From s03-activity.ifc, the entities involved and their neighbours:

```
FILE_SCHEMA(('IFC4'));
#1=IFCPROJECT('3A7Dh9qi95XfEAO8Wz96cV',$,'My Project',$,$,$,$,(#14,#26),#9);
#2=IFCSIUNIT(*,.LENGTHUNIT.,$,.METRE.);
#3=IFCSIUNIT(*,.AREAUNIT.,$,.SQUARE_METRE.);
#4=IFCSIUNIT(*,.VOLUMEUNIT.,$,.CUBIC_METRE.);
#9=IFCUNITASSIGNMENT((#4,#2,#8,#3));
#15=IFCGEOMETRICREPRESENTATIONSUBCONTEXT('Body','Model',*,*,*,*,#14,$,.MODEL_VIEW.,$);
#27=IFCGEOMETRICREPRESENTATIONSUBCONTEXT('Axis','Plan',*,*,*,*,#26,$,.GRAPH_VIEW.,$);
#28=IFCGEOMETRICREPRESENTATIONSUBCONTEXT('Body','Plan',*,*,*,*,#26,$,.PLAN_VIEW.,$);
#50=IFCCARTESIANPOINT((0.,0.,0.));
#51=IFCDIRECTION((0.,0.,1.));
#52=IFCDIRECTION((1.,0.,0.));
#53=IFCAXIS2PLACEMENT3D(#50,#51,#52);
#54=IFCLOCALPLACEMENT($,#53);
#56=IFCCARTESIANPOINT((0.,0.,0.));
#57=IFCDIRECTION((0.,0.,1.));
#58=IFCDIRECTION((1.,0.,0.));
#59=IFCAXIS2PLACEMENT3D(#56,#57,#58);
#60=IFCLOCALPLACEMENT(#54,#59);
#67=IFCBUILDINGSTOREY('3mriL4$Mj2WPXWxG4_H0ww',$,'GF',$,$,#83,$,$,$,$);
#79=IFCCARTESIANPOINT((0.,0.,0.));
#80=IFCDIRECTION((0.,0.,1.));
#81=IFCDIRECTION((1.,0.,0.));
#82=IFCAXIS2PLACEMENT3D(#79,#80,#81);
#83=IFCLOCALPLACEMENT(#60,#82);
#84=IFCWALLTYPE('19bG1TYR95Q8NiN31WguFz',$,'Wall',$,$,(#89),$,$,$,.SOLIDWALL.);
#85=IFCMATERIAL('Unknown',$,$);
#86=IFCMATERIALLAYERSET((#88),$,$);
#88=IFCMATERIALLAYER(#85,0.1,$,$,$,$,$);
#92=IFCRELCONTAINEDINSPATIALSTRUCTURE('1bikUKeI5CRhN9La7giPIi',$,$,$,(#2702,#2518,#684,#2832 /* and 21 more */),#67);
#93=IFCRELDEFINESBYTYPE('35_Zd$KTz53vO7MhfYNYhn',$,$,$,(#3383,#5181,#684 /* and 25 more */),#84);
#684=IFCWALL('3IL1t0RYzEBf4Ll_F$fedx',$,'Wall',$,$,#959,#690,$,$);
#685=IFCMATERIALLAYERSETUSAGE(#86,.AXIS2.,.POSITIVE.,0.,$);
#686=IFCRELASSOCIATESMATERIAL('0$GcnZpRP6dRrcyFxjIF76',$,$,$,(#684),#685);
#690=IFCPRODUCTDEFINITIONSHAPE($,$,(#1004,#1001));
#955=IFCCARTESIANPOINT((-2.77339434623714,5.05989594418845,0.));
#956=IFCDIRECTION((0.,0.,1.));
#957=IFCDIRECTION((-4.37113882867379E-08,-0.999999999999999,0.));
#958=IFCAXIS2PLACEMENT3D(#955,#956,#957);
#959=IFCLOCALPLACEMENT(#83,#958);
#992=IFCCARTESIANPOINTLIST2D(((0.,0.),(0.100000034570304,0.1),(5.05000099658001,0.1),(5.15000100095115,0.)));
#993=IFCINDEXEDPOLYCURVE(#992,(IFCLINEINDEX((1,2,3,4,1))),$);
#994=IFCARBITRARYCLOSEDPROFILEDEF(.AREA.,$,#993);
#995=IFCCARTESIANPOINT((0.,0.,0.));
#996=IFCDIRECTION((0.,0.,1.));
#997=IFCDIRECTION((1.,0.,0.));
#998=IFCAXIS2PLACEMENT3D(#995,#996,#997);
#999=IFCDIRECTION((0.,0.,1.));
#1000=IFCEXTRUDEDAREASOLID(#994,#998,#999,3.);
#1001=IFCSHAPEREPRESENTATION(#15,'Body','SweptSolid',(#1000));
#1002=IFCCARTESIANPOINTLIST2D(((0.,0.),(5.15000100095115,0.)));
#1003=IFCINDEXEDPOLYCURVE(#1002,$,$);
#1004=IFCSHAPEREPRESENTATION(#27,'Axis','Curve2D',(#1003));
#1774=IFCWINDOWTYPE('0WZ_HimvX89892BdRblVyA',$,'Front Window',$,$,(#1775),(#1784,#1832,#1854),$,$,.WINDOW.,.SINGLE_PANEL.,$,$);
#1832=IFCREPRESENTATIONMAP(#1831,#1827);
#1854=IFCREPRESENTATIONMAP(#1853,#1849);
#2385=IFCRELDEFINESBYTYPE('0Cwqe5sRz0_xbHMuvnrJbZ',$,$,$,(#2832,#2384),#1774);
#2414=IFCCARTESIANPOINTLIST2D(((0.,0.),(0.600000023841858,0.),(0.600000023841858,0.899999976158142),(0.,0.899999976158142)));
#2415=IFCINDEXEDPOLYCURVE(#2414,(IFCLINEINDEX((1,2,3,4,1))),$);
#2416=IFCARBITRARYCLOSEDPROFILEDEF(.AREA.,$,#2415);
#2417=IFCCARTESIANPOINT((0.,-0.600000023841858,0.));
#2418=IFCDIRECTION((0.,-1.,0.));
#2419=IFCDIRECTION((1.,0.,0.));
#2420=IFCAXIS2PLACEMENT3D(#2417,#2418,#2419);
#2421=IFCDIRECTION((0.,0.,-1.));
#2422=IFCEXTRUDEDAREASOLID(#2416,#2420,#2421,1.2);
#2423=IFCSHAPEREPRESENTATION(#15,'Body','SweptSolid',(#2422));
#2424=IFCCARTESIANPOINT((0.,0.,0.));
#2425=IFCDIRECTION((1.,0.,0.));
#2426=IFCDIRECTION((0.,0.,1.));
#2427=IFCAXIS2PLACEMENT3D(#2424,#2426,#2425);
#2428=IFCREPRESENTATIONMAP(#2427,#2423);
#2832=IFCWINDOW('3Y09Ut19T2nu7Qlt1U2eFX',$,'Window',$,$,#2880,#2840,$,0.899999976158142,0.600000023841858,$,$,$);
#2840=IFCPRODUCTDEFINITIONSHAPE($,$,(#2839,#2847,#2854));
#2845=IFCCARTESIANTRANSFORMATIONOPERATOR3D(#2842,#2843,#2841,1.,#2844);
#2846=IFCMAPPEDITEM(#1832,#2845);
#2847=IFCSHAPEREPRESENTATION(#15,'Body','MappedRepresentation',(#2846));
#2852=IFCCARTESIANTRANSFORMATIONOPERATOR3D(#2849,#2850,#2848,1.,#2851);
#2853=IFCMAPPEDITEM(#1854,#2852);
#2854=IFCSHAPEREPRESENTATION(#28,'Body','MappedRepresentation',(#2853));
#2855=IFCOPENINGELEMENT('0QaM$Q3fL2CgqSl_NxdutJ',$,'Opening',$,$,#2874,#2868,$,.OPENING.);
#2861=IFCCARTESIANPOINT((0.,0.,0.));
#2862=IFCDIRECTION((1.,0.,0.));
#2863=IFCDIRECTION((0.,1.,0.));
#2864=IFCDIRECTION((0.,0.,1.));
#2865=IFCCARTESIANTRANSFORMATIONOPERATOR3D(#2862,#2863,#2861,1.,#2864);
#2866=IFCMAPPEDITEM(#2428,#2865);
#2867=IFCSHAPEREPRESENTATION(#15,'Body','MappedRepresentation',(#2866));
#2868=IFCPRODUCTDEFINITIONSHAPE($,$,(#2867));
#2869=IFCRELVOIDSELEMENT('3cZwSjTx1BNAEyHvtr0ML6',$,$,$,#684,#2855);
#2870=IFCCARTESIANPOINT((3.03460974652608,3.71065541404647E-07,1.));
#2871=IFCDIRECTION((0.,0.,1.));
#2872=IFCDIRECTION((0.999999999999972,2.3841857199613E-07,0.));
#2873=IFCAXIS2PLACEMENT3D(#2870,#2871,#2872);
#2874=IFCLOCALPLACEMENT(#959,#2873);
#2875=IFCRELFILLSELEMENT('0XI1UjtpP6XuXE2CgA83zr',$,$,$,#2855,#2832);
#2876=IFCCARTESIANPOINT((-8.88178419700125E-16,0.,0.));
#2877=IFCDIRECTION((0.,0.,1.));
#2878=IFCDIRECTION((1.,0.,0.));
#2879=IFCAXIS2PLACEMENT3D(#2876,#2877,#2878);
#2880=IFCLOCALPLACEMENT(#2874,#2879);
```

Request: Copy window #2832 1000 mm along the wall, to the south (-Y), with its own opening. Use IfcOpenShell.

```python
import ifcopenshell
import ifcopenshell.api.feature
import ifcopenshell.api.geometry
import ifcopenshell.api.root
import ifcopenshell.geom
import ifcopenshell.util.element
import ifcopenshell.util.placement
import ifcopenshell.util.shape
import ifcopenshell.util.unit

model = ifcopenshell.open("s03-activity.ifc")
unit_scale = ifcopenshell.util.unit.calculate_unit_scale(model)
settings = ifcopenshell.geom.settings()


def volume(element):
    """Net volume in cubic metres, openings subtracted."""
    shape = ifcopenshell.geom.create_shape(settings, element)
    return ifcopenshell.util.shape.get_volume(shape.geometry)


window = model.by_guid("3Y09Ut19T2nu7Qlt1U2eFX")
opening = window.FillsVoids[0].RelatingOpeningElement
wall = opening.VoidsElements[0].RelatingBuildingElement
before = volume(wall)
shift = ifcopenshell.util.placement.get_local_placement(wall.ObjectPlacement)[:3, 0] * 1 / unit_scale

# copy_class copies the void relationship, type, container and properties, but no geometry.
new_opening = ifcopenshell.api.root.copy_class(model, product=opening)
new_opening.Representation = ifcopenshell.util.element.copy_deep(
    model, opening.Representation, exclude=["IfcGeometricRepresentationContext", "IfcRepresentationMap"]
)
new_window = ifcopenshell.api.root.copy_class(model, product=window)
new_window.Representation = ifcopenshell.util.element.copy_deep(
    model, window.Representation, exclude=["IfcGeometricRepresentationContext", "IfcRepresentationMap"]
)
ifcopenshell.api.feature.add_filling(model, opening=new_opening, element=new_window)

for old, new in ((opening, new_opening), (window, new_window)):
    matrix = ifcopenshell.util.placement.get_local_placement(old.ObjectPlacement)
    matrix[:3, 3] += shift
    ifcopenshell.api.geometry.edit_object_placement(model, product=new, matrix=matrix, is_si=False)

after = volume(wall)

print(f"wall volume {before:.3f} -> {after:.3f} m3")

model.write("s03-activity_v2.ifc")
```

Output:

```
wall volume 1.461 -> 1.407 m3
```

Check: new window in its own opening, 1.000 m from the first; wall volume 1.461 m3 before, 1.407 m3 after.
